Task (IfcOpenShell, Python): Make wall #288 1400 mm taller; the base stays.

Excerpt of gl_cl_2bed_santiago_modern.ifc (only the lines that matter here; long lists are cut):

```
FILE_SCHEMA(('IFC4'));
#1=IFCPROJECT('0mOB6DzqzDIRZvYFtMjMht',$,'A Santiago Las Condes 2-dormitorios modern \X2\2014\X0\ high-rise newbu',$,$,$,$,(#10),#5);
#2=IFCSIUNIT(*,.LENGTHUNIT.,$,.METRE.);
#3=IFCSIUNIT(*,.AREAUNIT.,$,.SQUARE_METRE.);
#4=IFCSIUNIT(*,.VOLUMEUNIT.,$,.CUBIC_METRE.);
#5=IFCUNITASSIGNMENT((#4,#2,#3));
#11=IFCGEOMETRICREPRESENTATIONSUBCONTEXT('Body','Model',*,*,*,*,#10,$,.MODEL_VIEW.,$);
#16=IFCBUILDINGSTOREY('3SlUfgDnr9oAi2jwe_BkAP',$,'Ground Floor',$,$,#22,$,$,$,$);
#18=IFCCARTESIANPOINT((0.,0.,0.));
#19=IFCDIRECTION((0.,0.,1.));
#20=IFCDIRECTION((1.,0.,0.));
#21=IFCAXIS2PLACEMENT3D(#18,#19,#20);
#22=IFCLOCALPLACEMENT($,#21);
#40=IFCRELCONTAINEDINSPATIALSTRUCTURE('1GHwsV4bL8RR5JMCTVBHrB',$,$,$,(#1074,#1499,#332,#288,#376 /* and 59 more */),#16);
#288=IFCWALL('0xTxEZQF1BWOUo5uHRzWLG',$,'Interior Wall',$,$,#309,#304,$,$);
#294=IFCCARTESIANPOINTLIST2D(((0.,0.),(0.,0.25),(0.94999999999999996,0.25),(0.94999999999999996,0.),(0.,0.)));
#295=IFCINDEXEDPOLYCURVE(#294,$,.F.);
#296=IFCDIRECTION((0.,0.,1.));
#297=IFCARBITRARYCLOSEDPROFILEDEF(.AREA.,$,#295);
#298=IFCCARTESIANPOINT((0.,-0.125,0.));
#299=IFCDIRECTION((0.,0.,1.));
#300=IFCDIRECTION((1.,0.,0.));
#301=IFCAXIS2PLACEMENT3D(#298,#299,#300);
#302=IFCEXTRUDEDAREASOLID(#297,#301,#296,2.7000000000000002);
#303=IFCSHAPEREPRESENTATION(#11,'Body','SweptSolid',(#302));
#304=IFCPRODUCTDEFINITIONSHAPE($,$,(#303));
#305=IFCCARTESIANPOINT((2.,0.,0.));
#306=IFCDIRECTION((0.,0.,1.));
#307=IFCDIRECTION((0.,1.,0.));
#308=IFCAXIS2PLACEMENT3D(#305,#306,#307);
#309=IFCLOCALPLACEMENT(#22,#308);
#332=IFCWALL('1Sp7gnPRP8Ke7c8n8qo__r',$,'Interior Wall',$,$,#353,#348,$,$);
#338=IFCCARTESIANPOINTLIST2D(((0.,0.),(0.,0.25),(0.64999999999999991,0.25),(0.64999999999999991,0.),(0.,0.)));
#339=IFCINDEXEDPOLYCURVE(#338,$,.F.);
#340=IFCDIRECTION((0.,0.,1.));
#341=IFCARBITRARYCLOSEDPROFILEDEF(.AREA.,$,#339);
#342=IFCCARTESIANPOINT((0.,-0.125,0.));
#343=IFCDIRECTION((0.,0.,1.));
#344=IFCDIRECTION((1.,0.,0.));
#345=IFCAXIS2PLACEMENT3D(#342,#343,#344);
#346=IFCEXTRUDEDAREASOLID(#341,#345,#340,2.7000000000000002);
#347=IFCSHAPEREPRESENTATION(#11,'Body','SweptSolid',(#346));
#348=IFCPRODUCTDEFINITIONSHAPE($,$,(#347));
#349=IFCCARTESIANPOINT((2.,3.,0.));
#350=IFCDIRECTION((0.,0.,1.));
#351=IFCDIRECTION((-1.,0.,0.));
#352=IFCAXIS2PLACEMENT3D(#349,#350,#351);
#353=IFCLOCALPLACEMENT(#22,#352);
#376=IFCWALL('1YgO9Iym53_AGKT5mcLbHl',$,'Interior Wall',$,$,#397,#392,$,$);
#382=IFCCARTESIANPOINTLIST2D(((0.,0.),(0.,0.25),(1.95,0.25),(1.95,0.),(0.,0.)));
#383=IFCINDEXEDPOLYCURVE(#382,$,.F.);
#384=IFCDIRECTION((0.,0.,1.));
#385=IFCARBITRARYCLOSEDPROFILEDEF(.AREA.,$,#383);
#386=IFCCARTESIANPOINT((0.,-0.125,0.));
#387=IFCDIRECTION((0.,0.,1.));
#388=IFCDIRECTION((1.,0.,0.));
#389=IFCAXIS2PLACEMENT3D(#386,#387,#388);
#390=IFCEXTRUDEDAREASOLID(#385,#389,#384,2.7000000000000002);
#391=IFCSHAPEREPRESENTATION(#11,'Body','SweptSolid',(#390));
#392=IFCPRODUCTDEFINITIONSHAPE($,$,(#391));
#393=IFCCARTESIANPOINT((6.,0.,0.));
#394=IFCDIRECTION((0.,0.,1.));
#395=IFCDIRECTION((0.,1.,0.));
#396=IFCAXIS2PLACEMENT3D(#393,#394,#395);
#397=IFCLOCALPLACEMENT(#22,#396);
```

```python
import ifcopenshell
import ifcopenshell.geom
import ifcopenshell.util.representation
import ifcopenshell.util.shape

model = ifcopenshell.open("gl_cl_2bed_santiago_modern.ifc")
settings = ifcopenshell.geom.settings()


def volume(element):
    """Net volume in cubic metres, openings subtracted."""
    shape = ifcopenshell.geom.create_shape(settings, element)
    return ifcopenshell.util.shape.get_volume(shape.geometry)


wall = model.by_id(288)
before = volume(wall)

body = ifcopenshell.util.representation.get_representation(wall, "Model", "Body")
solid = body.Items[0]
old_height = solid.Depth
solid.Depth += 1.4
after = volume(wall)

print(f"height {old_height:g} -> {solid.Depth:g}, volume {before:.3f} -> {after:.3f} m3")

model.write("gl_cl_2bed_santiago_modern-out.ifc")
```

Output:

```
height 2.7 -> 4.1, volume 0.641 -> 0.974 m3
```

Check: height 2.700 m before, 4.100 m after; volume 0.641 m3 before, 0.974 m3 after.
